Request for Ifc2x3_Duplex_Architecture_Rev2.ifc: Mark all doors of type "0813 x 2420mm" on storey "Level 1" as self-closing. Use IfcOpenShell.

First a look at what the model holds.

```python
import ifcopenshell
import ifcopenshell.util.element

model = ifcopenshell.open("Ifc2x3_Duplex_Architecture_Rev2.ifc")
print(model.schema)
storey = next(s for s in model.by_type("IfcBuildingStorey") if s.Name == "Level 1")
doors = [e for e in ifcopenshell.util.element.get_decomposition(storey) if e.is_a("IfcDoor")]
seen = {}
for e in doors:
    element_type = ifcopenshell.util.element.get_type(e)
    key = (element_type.Name if element_type != e and element_type else None, ifcopenshell.util.element.get_pset(e, "Pset_DoorCommon", "SelfClosing"))
    seen[key] = seen.get(key, 0) + 1
for (name, value), count in sorted(seen.items(), key=str):
    print(count, "x", name, "|", value)
```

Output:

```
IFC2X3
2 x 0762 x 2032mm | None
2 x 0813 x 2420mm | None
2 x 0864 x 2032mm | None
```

```python
import ifcopenshell
import ifcopenshell.api.pset
import ifcopenshell.util.element

model = ifcopenshell.open("Ifc2x3_Duplex_Architecture_Rev2.ifc")

storey = next(s for s in model.by_type("IfcBuildingStorey") if s.Name == "Level 1")
doors = [e for e in ifcopenshell.util.element.get_decomposition(storey) if e.is_a("IfcDoor")]

count = 0
for e in doors:
    element_type = ifcopenshell.util.element.get_type(e)
    if element_type in (None, e) or element_type.Name != "0813 x 2420mm":
        continue
    # add_pset returns the element's existing set when there is one.
    pset = ifcopenshell.api.pset.add_pset(model, product=e, name="Pset_DoorCommon")
    ifcopenshell.api.pset.edit_pset(model, pset=pset, properties={"SelfClosing": True})
    count += 1

print(count, "doors updated")

model.write("Ifc2x3_Duplex_Architecture_Rev2_edited.ifc")
```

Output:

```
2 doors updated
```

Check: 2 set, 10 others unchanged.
